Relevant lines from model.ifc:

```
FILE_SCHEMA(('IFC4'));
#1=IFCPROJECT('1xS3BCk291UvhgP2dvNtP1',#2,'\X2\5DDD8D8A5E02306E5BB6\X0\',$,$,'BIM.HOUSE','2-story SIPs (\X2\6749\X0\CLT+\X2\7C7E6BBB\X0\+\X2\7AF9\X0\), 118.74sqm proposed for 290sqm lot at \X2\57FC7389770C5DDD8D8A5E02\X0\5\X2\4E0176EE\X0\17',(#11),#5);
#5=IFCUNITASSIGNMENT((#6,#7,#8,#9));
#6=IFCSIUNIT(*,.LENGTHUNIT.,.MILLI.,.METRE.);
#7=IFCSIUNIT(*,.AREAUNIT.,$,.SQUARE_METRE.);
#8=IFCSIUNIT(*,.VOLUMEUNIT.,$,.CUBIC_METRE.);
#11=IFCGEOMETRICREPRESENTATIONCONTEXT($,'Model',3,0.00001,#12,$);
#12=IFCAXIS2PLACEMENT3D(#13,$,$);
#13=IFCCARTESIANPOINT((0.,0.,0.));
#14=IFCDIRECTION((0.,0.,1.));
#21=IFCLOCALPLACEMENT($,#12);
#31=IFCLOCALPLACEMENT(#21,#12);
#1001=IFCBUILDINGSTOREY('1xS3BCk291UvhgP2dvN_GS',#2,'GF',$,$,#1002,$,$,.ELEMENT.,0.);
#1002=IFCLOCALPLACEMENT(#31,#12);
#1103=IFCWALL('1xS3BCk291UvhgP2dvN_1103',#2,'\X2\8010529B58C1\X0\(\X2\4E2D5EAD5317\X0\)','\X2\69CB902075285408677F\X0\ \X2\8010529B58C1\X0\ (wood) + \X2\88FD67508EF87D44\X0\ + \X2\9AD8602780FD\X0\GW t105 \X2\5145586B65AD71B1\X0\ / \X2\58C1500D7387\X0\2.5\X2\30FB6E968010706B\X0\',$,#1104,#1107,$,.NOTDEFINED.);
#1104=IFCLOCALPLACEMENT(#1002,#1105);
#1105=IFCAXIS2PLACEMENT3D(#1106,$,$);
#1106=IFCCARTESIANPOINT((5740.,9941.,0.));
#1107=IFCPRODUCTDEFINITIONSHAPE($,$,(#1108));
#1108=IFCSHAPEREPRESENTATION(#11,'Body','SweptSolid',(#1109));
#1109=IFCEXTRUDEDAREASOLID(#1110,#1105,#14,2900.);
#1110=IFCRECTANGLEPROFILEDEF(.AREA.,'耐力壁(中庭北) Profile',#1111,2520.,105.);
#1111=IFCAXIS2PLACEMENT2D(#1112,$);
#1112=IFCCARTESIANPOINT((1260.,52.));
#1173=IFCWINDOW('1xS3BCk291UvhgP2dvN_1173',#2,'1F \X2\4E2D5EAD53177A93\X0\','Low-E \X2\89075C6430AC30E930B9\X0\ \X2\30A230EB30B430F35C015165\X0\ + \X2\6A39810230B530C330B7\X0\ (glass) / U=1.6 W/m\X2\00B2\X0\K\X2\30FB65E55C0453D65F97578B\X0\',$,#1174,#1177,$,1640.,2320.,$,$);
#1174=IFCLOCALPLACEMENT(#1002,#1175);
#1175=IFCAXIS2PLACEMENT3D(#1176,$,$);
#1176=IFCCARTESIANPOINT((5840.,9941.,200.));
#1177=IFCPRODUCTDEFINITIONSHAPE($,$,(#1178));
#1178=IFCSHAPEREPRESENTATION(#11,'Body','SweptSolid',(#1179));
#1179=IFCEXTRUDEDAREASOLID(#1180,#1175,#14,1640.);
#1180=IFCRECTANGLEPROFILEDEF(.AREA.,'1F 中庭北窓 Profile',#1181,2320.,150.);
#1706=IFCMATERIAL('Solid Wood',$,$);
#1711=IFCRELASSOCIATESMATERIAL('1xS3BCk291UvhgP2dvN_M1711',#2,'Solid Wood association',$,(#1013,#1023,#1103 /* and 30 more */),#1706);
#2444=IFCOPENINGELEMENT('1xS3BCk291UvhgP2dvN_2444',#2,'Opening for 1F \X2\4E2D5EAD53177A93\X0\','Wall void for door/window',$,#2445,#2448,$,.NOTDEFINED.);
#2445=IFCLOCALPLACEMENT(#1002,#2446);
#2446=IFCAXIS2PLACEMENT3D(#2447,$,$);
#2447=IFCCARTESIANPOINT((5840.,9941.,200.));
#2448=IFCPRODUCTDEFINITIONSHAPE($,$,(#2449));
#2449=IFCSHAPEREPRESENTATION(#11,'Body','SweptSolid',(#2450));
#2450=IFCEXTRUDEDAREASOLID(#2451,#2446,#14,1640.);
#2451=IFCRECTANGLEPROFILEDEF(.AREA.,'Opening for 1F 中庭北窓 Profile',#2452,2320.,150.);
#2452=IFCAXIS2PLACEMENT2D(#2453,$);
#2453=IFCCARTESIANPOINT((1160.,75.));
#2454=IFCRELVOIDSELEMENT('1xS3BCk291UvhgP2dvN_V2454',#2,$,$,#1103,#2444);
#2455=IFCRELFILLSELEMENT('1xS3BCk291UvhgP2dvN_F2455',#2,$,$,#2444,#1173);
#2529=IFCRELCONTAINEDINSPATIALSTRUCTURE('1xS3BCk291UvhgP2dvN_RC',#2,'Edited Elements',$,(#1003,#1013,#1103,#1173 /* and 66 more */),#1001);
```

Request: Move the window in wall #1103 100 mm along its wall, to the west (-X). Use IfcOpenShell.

```python
import ifcopenshell
import ifcopenshell.api.geometry
import ifcopenshell.util.placement
import ifcopenshell.util.unit

model = ifcopenshell.open("model.ifc")
unit_scale = ifcopenshell.util.unit.calculate_unit_scale(model)

window = model.by_guid("1xS3BCk291UvhgP2dvN_1173")
opening = window.FillsVoids[0].RelatingOpeningElement
wall = opening.VoidsElements[0].RelatingBuildingElement

wall_matrix = ifcopenshell.util.placement.get_local_placement(wall.ObjectPlacement)
shift = wall_matrix[:3, 0] * -0.1 / unit_scale
before = ifcopenshell.util.placement.get_local_placement(window.ObjectPlacement)[:3, 3].copy()

# The window is not placed relative to its opening, so move both.
for product in (opening, window):
    matrix = ifcopenshell.util.placement.get_local_placement(product.ObjectPlacement)
    matrix[:3, 3] += shift
    ifcopenshell.api.geometry.edit_object_placement(model, product=product, matrix=matrix, is_si=False)

after = ifcopenshell.util.placement.get_local_placement(window.ObjectPlacement)[:3, 3]
print("window moved by", (after - before).round(3) + 0.0)

model.write("model_updated.ifc")
```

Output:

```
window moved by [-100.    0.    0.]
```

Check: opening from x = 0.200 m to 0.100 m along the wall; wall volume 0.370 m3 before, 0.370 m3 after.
